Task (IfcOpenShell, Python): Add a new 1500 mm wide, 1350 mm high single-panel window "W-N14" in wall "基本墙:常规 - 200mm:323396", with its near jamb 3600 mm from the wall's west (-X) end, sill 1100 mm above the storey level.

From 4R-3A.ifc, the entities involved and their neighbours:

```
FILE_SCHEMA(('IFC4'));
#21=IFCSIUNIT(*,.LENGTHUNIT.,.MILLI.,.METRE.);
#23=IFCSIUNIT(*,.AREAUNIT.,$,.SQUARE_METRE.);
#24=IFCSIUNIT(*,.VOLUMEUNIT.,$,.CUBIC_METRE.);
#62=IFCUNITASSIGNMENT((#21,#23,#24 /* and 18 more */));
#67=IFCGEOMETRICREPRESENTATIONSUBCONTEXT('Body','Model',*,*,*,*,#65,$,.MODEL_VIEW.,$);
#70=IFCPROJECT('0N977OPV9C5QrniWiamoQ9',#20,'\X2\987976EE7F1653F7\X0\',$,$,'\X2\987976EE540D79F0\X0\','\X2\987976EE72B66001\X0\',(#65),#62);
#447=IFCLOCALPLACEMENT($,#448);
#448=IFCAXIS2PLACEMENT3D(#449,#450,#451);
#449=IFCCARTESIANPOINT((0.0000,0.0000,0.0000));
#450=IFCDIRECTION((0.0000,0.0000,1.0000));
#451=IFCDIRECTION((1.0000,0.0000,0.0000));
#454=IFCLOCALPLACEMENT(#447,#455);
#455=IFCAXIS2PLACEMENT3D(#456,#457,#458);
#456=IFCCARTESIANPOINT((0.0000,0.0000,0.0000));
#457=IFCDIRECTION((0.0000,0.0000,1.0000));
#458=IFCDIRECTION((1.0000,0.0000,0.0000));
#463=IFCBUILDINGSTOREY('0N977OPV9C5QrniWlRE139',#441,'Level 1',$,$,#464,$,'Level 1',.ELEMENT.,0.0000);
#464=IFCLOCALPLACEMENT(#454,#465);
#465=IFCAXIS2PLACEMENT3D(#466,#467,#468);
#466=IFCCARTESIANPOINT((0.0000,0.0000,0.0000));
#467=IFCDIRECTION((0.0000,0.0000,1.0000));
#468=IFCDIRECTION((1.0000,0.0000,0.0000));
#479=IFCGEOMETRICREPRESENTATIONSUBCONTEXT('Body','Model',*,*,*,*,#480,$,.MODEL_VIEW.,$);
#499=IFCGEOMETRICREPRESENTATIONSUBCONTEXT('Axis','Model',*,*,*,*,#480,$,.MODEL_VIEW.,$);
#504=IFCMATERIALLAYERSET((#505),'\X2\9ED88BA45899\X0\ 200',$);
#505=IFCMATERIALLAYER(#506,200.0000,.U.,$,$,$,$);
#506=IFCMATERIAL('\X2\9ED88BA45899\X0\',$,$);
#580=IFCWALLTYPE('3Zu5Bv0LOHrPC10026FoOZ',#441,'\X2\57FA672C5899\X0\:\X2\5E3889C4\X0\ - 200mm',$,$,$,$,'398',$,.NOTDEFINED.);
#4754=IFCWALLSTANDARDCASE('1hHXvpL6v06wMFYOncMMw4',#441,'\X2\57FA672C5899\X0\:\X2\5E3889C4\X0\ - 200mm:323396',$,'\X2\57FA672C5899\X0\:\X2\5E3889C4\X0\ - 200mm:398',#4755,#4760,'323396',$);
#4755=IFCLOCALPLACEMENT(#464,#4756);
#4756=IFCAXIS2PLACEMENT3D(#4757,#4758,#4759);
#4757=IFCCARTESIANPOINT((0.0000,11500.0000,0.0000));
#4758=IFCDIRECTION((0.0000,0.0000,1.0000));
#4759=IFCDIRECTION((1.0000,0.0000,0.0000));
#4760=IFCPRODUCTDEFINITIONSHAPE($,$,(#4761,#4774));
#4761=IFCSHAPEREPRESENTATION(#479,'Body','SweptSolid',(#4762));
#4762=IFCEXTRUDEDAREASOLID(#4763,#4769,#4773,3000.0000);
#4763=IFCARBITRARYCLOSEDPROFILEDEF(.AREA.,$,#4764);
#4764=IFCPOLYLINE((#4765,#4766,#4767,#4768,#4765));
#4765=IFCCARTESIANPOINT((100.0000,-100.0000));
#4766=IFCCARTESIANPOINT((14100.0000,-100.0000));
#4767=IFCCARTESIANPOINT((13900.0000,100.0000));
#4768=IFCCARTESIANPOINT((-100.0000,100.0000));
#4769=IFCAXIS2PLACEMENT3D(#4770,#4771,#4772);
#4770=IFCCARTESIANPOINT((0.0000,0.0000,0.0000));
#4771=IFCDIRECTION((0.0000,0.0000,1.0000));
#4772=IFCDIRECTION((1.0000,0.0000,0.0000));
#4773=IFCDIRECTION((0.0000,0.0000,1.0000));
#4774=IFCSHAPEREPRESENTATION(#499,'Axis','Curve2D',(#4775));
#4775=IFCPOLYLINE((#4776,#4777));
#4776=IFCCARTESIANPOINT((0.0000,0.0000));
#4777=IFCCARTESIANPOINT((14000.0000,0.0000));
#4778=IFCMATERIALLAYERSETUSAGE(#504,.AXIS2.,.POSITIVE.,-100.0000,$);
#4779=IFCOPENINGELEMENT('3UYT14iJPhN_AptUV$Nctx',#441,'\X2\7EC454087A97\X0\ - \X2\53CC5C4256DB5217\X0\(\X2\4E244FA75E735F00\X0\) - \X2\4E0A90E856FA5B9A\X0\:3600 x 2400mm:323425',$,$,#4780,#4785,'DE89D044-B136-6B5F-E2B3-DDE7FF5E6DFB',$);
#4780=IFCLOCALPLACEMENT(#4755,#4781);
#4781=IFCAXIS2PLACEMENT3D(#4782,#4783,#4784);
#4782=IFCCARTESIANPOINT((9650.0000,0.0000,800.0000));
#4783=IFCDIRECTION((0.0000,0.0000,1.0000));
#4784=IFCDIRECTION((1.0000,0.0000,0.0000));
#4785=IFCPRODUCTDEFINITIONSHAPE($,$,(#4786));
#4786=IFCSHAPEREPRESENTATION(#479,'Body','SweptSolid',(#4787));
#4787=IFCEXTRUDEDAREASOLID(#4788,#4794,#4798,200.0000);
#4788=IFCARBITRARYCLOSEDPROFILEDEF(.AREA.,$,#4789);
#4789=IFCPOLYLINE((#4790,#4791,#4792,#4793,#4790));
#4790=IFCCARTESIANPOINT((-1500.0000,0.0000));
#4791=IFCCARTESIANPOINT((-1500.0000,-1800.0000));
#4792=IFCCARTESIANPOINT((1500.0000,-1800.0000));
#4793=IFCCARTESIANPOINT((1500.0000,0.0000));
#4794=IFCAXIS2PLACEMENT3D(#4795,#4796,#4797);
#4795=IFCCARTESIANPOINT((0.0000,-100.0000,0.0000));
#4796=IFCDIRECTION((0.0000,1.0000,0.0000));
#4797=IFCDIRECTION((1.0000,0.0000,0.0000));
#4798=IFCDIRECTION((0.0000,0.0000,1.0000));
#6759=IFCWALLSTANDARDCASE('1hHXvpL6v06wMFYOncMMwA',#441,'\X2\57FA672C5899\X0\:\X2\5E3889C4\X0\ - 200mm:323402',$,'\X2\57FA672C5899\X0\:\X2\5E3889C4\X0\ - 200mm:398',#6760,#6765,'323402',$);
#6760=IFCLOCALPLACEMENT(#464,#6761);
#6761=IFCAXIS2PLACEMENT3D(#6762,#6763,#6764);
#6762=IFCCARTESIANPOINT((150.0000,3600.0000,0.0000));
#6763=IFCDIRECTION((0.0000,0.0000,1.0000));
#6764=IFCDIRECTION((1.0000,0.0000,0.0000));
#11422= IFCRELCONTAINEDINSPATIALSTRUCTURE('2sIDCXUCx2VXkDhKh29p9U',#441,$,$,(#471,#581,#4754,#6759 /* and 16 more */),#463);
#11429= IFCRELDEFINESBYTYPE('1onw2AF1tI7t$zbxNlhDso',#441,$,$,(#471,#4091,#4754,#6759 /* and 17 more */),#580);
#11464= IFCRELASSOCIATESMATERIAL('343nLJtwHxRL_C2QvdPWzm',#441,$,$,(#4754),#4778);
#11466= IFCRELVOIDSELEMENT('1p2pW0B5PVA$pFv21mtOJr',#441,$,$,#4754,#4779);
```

```python
import numpy as np
import ifcopenshell
import ifcopenshell.api.feature
import ifcopenshell.api.geometry
import ifcopenshell.api.root
import ifcopenshell.api.spatial
import ifcopenshell.geom
import ifcopenshell.util.element
import ifcopenshell.util.placement
import ifcopenshell.util.representation
import ifcopenshell.util.shape
import ifcopenshell.util.unit

model = ifcopenshell.open("4R-3A.ifc")
unit_scale = ifcopenshell.util.unit.calculate_unit_scale(model)
settings = ifcopenshell.geom.settings()


def volume(element):
    """Net volume in cubic metres, openings subtracted."""
    shape = ifcopenshell.geom.create_shape(settings, element)
    return ifcopenshell.util.shape.get_volume(shape.geometry)


wall = model.by_guid("1hHXvpL6v06wMFYOncMMw4")
storey = ifcopenshell.util.element.get_container(wall, ifc_class="IfcBuildingStorey")
context = ifcopenshell.util.representation.get_context(model, "Model", "Body", "MODEL_VIEW")
before = volume(wall)

width, height, from_end, sill = 1.5, 1.35, 3.6, 1.1  # metres

# The wall runs along its own X axis, and the end named is its -X end.
wall_shape = ifcopenshell.geom.create_shape(settings, wall)
x, y, z = ifcopenshell.util.shape.get_vertices(wall_shape.geometry).T
start = x.min() + from_end
face, thickness = float(y.min()), float(y.max() - y.min())
wall_matrix = ifcopenshell.util.placement.get_local_placement(wall.ObjectPlacement)
level = ifcopenshell.util.placement.get_local_placement(storey.ObjectPlacement)[2, 3]


def in_wall(x, y):
    """Placement at x, y metres in the wall's axes, at sill height."""
    matrix = wall_matrix.copy()
    matrix[:, 3] = wall_matrix @ np.array([x / unit_scale, y / unit_scale, 0.0, 1.0])
    matrix[2, 3] = level + sill / unit_scale
    return matrix


# Opening: a box that overshoots both wall faces by 50 mm.
opening = ifcopenshell.api.root.create_entity(model, ifc_class="IfcOpeningElement", predefined_type="OPENING")
box = ifcopenshell.api.geometry.add_wall_representation(
    model, context=context, length=width, height=height, thickness=thickness + 0.1
)
ifcopenshell.api.geometry.assign_representation(model, product=opening, representation=box)
ifcopenshell.api.geometry.edit_object_placement(model, product=opening, matrix=in_wall(start, face - 0.05), is_si=False)
ifcopenshell.api.feature.add_feature(model, feature=opening, element=wall)

window = ifcopenshell.api.root.create_entity(model, ifc_class="IfcWindow", name="W-N14", predefined_type="WINDOW")
window.OverallWidth, window.OverallHeight = width / unit_scale, height / unit_scale
window.PartitioningType = "SINGLE_PANEL"
body = ifcopenshell.api.geometry.add_window_representation(
    model,
    context=context,
    overall_width=window.OverallWidth,
    overall_height=window.OverallHeight,
    partition_type="SINGLE_PANEL",
)
ifcopenshell.api.geometry.assign_representation(model, product=window, representation=body)
ifcopenshell.api.spatial.assign_container(model, products=[window], relating_structure=storey)
ifcopenshell.api.feature.add_filling(model, opening=opening, element=window)

# Centre the window in the wall's thickness.
ifcopenshell.api.geometry.edit_object_placement(model, product=window, matrix=in_wall(start, face), is_si=False)
window_shape = ifcopenshell.geom.create_shape(settings, window)
depth = ifcopenshell.util.shape.get_vertices(window_shape.geometry)[:, 1]
offset = face + thickness / 2 - (depth.min() + depth.max()) / 2
ifcopenshell.api.geometry.edit_object_placement(model, product=window, matrix=in_wall(start, offset), is_si=False)

after = volume(wall)

print(f"wall volume {before:.3f} -> {after:.3f} m3")

model.write("4R-3A-out.ifc")
```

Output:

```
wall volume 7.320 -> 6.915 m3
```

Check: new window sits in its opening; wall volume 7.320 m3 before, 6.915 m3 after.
